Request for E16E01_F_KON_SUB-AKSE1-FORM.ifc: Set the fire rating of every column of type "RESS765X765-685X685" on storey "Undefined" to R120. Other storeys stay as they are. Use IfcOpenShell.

First a look at what the model holds.

```python
import ifcopenshell
import ifcopenshell.util.element

model = ifcopenshell.open("E16E01_F_KON_SUB-AKSE1-FORM.ifc")
print(model.schema)
storey = next(s for s in model.by_type("IfcBuildingStorey") if s.Name == "Undefined")
columns = [e for e in ifcopenshell.util.element.get_decomposition(storey) if e.is_a("IfcColumn")]
seen = {}
for e in columns:
    element_type = ifcopenshell.util.element.get_type(e)
    key = (element_type.Name if element_type != e and element_type else None, ifcopenshell.util.element.get_pset(e, "Pset_ColumnCommon", "FireRating"))
    seen[key] = seen.get(key, 0) + 1
for (name, value), count in sorted(seen.items(), key=str):
    print(count, "x", name, "|", value)
```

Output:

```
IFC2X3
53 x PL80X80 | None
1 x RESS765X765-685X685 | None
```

```python
import ifcopenshell
import ifcopenshell.api.pset
import ifcopenshell.util.element

model = ifcopenshell.open("E16E01_F_KON_SUB-AKSE1-FORM.ifc")

storey = next(s for s in model.by_type("IfcBuildingStorey") if s.Name == "Undefined")
columns = [e for e in ifcopenshell.util.element.get_decomposition(storey) if e.is_a("IfcColumn")]

count = 0
for e in columns:
    element_type = ifcopenshell.util.element.get_type(e)
    if element_type in (None, e) or element_type.Name != "RESS765X765-685X685":
        continue
    # add_pset returns the element's existing set when there is one.
    pset = ifcopenshell.api.pset.add_pset(model, product=e, name="Pset_ColumnCommon")
    ifcopenshell.api.pset.edit_pset(model, pset=pset, properties={"FireRating": "R120"})
    count += 1

print(count, "columns updated")

model.write("E16E01_F_KON_SUB-AKSE1-FORM_rev.ifc")
```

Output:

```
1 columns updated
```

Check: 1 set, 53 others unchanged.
